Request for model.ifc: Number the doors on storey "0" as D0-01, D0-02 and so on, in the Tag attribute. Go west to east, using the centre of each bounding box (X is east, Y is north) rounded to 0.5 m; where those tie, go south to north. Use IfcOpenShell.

First a look at what the model holds.

```python
import ifcopenshell
import ifcopenshell.util.element
import ifcopenshell.util.placement

model = ifcopenshell.open("model.ifc")
print(model.schema)
storey = next(s for s in model.by_type("IfcBuildingStorey") if s.Name == "0")
doors = [e for e in ifcopenshell.util.element.get_decomposition(storey) if e.is_a("IfcDoor")]
for e in sorted(doors, key=lambda e: e.id()):
    origin = ifcopenshell.util.placement.get_local_placement(e.ObjectPlacement)[:3, 3]
    print(e.id(), e.Tag, e.Name, origin.round(2) + 0.0, sep=" | ")
```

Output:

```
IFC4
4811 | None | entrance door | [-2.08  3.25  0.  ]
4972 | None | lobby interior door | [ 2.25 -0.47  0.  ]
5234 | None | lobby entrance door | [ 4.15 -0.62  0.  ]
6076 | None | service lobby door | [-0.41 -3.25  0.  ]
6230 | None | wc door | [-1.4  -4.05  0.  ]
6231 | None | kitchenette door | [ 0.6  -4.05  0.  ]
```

```python
import ifcopenshell
import ifcopenshell.geom
import ifcopenshell.util.element
import ifcopenshell.util.shape

model = ifcopenshell.open("model.ifc")
settings = ifcopenshell.geom.settings()
settings.set("use-world-coords", True)


def centre(element):
    shape = ifcopenshell.geom.create_shape(settings, element)
    return ifcopenshell.util.shape.get_bbox_centroid(shape.geometry)


storey = next(s for s in model.by_type("IfcBuildingStorey") if s.Name == "0")
doors = [e for e in ifcopenshell.util.element.get_decomposition(storey) if e.is_a("IfcDoor")]

# Insertion points can sit at a corner or the storey origin, so sort by the geometry (in metres).
centres = {e: centre(e) for e in doors}
doors.sort(key=lambda e: (round(centres[e][0] / 0.5), centres[e][1]))

for i, e in enumerate(doors, start=1):
    number = f"D0-{i:02d}"
    e.Tag = number
    print(e.id(), number)

model.write("model_edited.ifc")
```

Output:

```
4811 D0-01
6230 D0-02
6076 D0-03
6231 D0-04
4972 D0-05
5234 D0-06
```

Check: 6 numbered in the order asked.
